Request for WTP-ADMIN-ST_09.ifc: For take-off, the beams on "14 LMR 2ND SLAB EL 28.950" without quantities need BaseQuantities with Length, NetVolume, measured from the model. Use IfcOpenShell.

First a look at what the model holds.

```python
import ifcopenshell
import ifcopenshell.util.element
import ifcopenshell.util.unit

model = ifcopenshell.open("WTP-ADMIN-ST_09.ifc")
print(model.schema)
for unit_type in ("LENGTHUNIT", "AREAUNIT", "VOLUMEUNIT"):
    print(unit_type, ifcopenshell.util.unit.calculate_unit_scale(model, unit_type))
storey = next(s for s in model.by_type("IfcBuildingStorey") if s.Name == "14 LMR 2ND SLAB EL 28.950")
beams = [e for e in ifcopenshell.util.element.get_decomposition(storey) if e.is_a("IfcBeam")]
for e in sorted(beams, key=lambda e: e.id()):
    print(e.id(), e.is_a(), e.Name, list(ifcopenshell.util.element.get_psets(e, qtos_only=True)), sep=" | ")
```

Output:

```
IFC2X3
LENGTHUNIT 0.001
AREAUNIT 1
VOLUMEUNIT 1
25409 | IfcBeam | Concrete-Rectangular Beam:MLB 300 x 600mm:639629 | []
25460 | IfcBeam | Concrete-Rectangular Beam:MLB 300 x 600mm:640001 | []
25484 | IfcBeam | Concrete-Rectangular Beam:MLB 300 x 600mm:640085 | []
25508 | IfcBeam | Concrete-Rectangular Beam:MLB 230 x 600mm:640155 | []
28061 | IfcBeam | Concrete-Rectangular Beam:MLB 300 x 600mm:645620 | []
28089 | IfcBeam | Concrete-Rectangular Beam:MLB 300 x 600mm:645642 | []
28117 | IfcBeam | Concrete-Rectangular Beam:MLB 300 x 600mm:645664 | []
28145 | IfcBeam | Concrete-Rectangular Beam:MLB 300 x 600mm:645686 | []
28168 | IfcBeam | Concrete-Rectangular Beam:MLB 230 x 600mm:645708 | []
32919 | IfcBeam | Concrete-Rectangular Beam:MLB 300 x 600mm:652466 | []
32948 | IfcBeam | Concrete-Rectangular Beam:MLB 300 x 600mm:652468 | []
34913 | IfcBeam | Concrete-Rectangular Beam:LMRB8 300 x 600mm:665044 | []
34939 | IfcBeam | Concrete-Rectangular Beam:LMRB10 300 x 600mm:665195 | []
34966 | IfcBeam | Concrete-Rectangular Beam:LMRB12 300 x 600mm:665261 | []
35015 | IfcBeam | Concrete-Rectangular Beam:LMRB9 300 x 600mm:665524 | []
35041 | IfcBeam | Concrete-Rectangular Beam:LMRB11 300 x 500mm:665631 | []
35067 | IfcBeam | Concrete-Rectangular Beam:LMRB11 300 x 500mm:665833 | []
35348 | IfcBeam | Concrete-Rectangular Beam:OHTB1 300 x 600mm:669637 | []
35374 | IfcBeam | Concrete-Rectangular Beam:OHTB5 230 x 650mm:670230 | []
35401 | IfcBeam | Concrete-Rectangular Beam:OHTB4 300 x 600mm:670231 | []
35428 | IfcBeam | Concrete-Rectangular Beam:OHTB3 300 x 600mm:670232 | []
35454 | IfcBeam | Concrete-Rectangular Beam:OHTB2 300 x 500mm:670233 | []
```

```python
import ifcopenshell
import ifcopenshell.api.pset
import ifcopenshell.geom
import ifcopenshell.util.element
import ifcopenshell.util.shape
import ifcopenshell.util.unit

model = ifcopenshell.open("WTP-ADMIN-ST_09.ifc")
unit_scale = ifcopenshell.util.unit.calculate_unit_scale(model)
volume_scale = ifcopenshell.util.unit.calculate_unit_scale(model, "VOLUMEUNIT")
settings = ifcopenshell.geom.settings()

storey = next(s for s in model.by_type("IfcBuildingStorey") if s.Name == "14 LMR 2ND SLAB EL 28.950")
beams = [e for e in ifcopenshell.util.element.get_decomposition(storey) if e.is_a("IfcBeam")]

for e in sorted(beams, key=lambda e: e.id()):
    if ifcopenshell.util.element.get_psets(e, qtos_only=True, should_inherit=False):
        continue
    # Geometry comes back in metres, in the element's own axes.
    shape = ifcopenshell.geom.create_shape(settings, e)
    values = {
        "Length": ifcopenshell.util.shape.get_max_xyz(shape.geometry) / unit_scale,
        "NetVolume": ifcopenshell.util.shape.get_volume(shape.geometry) / volume_scale,
    }
    qto = ifcopenshell.api.pset.add_qto(model, product=e, name="BaseQuantities")
    ifcopenshell.api.pset.edit_qto(model, qto=qto, properties=values)
    print(e.id(), {k: round(v, 3) for k, v in values.items()})

model.write("WTP-ADMIN-ST_09_updated.ifc")
```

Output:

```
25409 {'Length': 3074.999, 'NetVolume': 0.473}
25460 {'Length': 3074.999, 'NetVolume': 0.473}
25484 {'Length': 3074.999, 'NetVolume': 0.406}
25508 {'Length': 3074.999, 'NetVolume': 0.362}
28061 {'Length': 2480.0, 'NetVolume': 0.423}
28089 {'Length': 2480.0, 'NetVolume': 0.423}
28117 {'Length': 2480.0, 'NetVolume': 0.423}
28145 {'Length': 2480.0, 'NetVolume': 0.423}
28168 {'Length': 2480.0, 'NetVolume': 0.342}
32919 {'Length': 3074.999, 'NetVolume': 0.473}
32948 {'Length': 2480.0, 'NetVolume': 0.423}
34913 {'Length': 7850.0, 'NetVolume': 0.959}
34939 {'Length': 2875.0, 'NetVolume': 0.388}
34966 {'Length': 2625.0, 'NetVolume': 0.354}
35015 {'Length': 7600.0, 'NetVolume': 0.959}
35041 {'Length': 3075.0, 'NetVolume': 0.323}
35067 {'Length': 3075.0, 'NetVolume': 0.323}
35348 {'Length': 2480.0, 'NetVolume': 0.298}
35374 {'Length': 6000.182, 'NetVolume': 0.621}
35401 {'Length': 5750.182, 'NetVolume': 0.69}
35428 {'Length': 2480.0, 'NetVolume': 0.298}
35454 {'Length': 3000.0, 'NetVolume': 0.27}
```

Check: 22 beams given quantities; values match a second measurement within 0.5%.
